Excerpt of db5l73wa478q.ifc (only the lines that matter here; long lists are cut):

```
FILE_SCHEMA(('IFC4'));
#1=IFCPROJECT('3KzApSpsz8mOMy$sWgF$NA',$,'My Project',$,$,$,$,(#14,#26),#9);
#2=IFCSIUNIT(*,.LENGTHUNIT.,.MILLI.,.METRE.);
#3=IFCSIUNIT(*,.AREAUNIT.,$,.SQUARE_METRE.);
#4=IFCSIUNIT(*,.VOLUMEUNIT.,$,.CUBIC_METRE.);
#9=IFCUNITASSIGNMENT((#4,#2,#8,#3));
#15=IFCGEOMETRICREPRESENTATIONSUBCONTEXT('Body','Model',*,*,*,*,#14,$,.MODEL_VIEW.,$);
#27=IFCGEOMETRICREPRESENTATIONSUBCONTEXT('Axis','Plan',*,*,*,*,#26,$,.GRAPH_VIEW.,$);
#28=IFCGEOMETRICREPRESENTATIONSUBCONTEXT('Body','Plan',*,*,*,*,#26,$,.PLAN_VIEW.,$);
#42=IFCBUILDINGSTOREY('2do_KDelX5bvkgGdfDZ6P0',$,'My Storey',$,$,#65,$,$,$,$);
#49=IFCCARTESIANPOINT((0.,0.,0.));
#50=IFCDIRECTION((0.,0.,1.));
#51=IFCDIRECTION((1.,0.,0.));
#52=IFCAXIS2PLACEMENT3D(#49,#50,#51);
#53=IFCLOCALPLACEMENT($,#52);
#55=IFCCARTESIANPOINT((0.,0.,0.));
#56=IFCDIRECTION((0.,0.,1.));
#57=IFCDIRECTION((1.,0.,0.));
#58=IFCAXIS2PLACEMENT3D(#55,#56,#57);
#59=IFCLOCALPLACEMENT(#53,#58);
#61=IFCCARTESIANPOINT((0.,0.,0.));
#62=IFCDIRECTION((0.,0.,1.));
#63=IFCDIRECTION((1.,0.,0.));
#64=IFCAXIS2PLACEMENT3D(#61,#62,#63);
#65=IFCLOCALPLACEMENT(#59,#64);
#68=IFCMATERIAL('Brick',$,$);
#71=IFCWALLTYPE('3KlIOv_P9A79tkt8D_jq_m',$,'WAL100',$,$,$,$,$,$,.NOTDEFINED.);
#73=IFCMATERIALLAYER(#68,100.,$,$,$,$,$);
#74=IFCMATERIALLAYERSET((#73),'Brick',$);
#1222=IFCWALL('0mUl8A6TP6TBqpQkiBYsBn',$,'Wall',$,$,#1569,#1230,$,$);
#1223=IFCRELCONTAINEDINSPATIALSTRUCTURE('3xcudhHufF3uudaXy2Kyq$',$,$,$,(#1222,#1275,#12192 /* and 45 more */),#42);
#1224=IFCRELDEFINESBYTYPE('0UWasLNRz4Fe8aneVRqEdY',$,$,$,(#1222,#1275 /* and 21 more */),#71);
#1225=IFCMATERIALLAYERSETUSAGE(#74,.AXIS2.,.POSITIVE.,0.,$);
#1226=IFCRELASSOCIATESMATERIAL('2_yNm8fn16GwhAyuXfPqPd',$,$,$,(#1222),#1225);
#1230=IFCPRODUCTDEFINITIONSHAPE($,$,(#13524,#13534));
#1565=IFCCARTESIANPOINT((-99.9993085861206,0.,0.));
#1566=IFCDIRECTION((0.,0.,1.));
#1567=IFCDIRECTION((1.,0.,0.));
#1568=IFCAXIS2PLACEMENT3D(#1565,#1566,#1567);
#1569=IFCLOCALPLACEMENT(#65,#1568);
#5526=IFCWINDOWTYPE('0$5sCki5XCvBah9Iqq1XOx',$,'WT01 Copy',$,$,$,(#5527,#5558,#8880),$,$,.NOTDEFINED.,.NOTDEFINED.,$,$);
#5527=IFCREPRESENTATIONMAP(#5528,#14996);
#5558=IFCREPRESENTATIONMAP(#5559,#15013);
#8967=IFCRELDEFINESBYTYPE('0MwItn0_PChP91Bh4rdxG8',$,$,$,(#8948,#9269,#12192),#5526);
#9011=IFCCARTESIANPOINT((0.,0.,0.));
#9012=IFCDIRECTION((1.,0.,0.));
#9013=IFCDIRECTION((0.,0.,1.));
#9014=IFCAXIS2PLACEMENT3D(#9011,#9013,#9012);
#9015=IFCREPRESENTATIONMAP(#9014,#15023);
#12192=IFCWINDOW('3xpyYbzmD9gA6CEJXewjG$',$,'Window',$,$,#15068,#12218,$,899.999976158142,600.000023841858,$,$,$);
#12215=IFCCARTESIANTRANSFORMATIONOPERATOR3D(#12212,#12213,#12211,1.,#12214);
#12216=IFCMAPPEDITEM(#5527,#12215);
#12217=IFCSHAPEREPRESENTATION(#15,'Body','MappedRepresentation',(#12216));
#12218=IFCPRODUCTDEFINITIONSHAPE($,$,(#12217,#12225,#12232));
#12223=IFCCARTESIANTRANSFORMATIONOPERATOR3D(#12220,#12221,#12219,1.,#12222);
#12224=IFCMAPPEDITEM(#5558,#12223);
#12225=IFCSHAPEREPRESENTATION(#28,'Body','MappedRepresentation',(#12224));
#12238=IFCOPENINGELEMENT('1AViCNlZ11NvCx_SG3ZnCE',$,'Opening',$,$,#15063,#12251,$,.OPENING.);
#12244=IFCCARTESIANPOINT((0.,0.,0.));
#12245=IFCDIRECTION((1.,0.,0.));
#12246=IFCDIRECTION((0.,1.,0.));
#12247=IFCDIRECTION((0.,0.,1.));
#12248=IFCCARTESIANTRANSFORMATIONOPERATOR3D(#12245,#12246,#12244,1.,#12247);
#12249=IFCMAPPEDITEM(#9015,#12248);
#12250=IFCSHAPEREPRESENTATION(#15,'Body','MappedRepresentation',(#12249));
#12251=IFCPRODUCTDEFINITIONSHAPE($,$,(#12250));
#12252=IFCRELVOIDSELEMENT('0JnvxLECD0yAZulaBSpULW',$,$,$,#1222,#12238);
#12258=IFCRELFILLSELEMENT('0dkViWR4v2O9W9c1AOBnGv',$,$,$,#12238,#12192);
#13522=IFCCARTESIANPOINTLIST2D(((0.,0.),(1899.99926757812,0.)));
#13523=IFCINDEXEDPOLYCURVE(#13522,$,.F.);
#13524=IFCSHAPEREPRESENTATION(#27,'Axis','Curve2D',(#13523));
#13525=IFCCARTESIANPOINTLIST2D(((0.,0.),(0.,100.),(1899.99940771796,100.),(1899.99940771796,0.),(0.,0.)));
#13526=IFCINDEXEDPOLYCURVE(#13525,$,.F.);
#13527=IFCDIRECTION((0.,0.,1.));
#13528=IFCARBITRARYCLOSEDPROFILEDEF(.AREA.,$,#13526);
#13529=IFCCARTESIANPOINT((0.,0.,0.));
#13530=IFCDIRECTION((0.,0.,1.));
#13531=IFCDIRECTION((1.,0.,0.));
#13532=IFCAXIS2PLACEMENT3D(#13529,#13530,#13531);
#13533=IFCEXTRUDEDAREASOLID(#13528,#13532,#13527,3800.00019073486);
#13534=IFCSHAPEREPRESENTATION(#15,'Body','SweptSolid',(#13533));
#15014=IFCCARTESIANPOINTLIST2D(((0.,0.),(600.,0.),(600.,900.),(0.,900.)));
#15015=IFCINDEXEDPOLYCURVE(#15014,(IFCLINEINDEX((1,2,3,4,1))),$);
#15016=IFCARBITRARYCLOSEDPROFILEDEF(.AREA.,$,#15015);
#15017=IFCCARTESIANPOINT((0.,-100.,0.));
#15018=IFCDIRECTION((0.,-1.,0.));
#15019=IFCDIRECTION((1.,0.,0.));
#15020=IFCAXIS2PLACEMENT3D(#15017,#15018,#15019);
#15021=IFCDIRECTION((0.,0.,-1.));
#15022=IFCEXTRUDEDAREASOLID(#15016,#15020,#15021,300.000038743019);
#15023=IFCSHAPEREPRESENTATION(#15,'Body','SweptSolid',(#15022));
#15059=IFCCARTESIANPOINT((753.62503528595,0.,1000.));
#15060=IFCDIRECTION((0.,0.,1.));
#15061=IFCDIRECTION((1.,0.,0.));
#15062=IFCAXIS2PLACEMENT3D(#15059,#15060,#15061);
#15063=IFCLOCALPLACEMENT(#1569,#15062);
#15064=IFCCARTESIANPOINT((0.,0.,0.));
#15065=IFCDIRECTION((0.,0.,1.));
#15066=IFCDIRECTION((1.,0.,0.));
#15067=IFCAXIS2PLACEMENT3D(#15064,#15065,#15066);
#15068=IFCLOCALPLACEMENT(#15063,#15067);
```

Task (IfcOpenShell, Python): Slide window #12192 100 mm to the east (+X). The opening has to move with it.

```python
import ifcopenshell
import ifcopenshell.api.geometry
import ifcopenshell.util.placement

model = ifcopenshell.open("db5l73wa478q.ifc")

window = model.by_id(12192)
opening = window.FillsVoids[0].RelatingOpeningElement
wall = opening.VoidsElements[0].RelatingBuildingElement

wall_matrix = ifcopenshell.util.placement.get_local_placement(wall.ObjectPlacement)
shift = wall_matrix[:3, 0] * 100.0
before = ifcopenshell.util.placement.get_local_placement(window.ObjectPlacement)[:3, 3].copy()

# The window is placed relative to its opening, so it follows when the opening moves.
matrix = ifcopenshell.util.placement.get_local_placement(opening.ObjectPlacement)
matrix[:3, 3] += shift
ifcopenshell.api.geometry.edit_object_placement(
    model, product=opening, matrix=matrix, is_si=False, should_transform_children=True
)

after = ifcopenshell.util.placement.get_local_placement(window.ObjectPlacement)[:3, 3]
print("window moved by", (after - before).round(3) + 0.0)

model.write("db5l73wa478q_edited.ifc")
```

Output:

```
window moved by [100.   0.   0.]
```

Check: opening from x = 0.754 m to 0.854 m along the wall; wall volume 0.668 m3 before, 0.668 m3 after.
